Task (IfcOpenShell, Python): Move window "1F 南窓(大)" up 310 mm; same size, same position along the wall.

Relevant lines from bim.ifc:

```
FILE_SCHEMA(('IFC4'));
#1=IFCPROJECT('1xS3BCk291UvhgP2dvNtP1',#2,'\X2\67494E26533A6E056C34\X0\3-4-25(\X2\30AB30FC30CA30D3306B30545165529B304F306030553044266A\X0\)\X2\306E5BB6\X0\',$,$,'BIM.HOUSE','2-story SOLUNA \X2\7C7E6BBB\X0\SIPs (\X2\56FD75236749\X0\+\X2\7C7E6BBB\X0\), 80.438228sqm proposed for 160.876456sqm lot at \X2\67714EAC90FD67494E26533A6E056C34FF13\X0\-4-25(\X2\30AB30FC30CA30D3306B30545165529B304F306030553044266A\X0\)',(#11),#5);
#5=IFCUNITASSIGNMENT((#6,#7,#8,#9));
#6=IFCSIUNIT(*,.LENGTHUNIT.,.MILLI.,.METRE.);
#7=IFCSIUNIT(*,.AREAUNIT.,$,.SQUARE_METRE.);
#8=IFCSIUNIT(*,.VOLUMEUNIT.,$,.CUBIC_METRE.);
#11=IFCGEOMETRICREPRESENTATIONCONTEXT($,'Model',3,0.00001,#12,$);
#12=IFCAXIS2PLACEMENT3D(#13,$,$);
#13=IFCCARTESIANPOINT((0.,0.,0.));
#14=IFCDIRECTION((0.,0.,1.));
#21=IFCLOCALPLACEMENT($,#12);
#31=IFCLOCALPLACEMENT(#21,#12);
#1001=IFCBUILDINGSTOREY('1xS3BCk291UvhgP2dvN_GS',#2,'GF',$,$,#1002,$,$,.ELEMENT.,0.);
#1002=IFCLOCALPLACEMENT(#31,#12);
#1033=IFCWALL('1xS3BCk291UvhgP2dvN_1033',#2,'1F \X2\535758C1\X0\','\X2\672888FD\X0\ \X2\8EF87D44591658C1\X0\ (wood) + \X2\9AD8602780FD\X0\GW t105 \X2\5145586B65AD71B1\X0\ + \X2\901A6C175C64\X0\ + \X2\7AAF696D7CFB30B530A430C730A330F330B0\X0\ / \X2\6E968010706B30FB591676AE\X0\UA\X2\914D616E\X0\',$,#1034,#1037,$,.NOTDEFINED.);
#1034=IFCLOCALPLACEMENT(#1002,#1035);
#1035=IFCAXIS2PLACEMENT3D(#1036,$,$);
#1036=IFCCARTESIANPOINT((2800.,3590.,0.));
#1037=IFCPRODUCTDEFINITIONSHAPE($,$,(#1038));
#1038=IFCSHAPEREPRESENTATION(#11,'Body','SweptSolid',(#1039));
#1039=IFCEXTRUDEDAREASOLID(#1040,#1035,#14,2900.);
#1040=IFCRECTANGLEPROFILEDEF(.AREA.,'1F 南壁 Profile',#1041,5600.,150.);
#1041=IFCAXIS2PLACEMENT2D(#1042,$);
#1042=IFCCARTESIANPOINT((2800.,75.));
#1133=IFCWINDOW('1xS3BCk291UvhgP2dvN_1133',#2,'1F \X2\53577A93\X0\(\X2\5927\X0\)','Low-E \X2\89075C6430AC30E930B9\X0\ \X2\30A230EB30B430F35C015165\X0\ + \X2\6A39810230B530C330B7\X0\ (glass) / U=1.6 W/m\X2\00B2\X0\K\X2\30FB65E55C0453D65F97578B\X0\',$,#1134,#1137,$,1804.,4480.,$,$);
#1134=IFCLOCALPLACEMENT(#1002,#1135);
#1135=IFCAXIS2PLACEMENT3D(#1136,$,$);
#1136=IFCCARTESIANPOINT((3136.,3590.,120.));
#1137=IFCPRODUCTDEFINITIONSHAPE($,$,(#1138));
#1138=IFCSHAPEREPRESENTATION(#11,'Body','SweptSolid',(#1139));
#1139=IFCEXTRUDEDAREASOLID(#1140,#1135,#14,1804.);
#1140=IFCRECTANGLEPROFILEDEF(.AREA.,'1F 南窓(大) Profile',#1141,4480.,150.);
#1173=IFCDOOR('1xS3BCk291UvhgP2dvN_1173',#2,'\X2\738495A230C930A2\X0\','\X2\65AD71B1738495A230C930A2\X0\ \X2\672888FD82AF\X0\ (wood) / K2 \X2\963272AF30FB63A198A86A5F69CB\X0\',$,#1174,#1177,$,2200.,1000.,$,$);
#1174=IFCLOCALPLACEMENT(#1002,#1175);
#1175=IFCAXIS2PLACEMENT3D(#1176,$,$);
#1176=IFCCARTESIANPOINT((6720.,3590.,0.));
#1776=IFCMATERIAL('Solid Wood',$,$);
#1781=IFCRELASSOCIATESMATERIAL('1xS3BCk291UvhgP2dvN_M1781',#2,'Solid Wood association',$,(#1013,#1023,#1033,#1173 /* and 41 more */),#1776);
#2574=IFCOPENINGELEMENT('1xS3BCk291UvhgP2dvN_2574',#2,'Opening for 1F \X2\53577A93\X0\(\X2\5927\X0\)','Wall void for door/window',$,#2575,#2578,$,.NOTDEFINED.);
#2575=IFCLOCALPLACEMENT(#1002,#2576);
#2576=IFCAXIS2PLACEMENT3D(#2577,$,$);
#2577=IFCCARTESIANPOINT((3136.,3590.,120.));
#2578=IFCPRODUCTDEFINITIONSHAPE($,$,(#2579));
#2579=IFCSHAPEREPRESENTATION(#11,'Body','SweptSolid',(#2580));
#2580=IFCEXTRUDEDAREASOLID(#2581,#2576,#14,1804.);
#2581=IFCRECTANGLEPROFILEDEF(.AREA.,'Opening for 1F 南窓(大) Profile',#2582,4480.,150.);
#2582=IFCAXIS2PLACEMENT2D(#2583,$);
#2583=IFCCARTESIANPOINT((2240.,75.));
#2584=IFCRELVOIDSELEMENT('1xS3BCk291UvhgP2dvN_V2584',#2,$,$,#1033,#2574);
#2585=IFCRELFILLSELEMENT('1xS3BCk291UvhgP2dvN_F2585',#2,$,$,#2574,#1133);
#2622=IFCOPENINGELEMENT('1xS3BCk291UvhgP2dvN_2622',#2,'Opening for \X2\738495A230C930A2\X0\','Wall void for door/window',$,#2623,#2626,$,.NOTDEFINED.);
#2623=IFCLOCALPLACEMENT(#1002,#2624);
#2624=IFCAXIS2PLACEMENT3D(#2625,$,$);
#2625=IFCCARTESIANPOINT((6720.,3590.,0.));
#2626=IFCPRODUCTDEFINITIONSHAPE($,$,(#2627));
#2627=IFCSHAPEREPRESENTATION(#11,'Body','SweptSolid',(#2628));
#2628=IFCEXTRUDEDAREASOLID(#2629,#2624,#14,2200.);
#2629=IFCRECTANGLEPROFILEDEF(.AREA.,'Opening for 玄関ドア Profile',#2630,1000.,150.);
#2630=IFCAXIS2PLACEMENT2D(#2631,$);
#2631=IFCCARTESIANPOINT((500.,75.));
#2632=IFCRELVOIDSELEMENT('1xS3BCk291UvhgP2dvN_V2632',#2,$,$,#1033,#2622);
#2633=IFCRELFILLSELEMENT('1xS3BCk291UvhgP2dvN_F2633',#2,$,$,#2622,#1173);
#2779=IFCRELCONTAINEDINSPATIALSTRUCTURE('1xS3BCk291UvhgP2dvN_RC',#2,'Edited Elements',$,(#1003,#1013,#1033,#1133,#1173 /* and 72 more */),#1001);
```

```python
import numpy as np
import ifcopenshell
import ifcopenshell.api.geometry
import ifcopenshell.util.placement
import ifcopenshell.util.unit

model = ifcopenshell.open("bim.ifc")
unit_scale = ifcopenshell.util.unit.calculate_unit_scale(model)

window = model.by_id(1133)
opening = window.FillsVoids[0].RelatingOpeningElement
dz = 0.31 / unit_scale

shift = np.array([0.0, 0.0, dz])
# The window is not placed relative to its opening, so move both.
for product in (opening, window):
    matrix = ifcopenshell.util.placement.get_local_placement(product.ObjectPlacement)
    matrix[:3, 3] += shift
    ifcopenshell.api.geometry.edit_object_placement(model, product=product, matrix=matrix, is_si=False)

print(f"moved by {dz * unit_scale:+.3f} m")

model.write("bim-out.ifc")
```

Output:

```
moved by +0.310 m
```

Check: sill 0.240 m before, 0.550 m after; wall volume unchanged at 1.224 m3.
